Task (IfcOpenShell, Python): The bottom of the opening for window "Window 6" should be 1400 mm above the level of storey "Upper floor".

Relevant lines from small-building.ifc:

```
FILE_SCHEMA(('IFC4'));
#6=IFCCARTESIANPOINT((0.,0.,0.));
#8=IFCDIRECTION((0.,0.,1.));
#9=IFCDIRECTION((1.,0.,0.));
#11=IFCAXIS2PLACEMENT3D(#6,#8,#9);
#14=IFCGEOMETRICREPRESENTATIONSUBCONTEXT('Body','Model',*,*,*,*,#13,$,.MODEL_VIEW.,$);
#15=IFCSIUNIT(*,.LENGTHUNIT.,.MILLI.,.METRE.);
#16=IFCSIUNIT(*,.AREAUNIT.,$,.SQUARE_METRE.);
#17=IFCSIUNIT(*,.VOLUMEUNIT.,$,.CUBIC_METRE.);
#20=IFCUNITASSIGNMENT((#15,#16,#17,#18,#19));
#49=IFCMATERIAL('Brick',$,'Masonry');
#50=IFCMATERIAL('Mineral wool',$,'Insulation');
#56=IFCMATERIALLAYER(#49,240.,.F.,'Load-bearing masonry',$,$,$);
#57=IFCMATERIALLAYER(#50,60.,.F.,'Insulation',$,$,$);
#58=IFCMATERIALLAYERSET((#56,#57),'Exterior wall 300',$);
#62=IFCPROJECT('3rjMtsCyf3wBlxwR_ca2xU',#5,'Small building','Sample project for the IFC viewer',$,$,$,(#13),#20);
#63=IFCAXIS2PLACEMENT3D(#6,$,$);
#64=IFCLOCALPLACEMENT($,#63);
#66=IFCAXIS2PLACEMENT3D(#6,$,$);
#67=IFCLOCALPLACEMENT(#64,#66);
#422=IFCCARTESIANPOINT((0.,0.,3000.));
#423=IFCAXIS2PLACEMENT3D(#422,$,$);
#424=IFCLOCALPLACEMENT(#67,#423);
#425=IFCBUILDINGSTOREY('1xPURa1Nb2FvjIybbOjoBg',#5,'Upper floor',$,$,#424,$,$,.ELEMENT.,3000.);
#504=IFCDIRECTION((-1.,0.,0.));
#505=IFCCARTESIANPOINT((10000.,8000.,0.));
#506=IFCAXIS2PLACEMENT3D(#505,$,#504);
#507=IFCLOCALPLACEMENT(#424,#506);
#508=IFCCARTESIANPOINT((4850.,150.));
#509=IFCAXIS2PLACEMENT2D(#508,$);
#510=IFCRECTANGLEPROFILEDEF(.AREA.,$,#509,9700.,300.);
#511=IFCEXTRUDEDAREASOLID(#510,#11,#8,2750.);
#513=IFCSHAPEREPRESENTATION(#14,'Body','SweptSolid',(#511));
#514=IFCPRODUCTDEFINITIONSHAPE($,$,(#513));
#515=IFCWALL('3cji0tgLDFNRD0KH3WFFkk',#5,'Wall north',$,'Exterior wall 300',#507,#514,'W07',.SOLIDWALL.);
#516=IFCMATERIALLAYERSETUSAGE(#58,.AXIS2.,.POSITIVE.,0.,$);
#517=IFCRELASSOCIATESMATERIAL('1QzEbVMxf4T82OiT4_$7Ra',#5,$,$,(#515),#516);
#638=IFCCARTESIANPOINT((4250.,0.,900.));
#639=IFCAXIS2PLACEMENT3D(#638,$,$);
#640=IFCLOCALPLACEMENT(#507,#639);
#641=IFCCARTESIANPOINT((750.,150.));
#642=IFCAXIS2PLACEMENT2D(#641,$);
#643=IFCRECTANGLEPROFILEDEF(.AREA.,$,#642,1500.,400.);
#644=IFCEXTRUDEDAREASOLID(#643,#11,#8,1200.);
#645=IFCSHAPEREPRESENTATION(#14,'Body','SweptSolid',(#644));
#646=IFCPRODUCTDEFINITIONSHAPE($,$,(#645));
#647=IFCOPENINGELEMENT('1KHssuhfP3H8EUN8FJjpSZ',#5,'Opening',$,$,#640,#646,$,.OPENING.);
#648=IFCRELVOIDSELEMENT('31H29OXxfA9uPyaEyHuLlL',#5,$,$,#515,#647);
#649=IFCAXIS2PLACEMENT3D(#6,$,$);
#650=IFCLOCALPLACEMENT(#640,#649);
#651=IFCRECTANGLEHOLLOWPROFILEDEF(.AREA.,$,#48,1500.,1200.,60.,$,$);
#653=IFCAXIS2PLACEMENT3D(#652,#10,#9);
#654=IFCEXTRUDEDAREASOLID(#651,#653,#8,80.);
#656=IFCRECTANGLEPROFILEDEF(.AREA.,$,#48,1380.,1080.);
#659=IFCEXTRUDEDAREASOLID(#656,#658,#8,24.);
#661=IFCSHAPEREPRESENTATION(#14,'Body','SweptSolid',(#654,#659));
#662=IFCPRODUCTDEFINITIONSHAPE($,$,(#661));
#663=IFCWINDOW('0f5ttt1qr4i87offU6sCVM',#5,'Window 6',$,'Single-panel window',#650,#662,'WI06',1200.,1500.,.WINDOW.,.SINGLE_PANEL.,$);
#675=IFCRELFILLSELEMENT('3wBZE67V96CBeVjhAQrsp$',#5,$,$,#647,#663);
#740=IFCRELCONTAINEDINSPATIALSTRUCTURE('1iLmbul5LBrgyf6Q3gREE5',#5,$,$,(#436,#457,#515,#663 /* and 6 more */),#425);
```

```python
import numpy as np
import ifcopenshell
import ifcopenshell.api.geometry
import ifcopenshell.geom
import ifcopenshell.util.element
import ifcopenshell.util.placement
import ifcopenshell.util.shape
import ifcopenshell.util.unit

model = ifcopenshell.open("small-building.ifc")
unit_scale = ifcopenshell.util.unit.calculate_unit_scale(model)

window = model.by_guid("0f5ttt1qr4i87offU6sCVM")
opening = window.FillsVoids[0].RelatingOpeningElement
storey = ifcopenshell.util.element.get_container(window, ifc_class="IfcBuildingStorey")
level = ifcopenshell.util.placement.get_local_placement(storey.ObjectPlacement)[2, 3]

# The opening's origin need not be at the sill, so measure its lowest point.
shape = ifcopenshell.geom.create_shape(ifcopenshell.geom.settings(), opening)
bottom = ifcopenshell.util.shape.get_shape_bottom_elevation(shape, shape.geometry) / unit_scale
dz = level + 1400.0 - bottom

shift = np.array([0.0, 0.0, dz])
# The window is placed relative to its opening, so it follows when the opening moves.
matrix = ifcopenshell.util.placement.get_local_placement(opening.ObjectPlacement)
matrix[:3, 3] += shift
ifcopenshell.api.geometry.edit_object_placement(
    model, product=opening, matrix=matrix, is_si=False, should_transform_children=True
)

print(f"moved by {dz * unit_scale:+.3f} m")

model.write("small-building_edited.ifc")
```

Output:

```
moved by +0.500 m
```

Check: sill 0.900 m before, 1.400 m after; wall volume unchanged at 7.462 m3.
